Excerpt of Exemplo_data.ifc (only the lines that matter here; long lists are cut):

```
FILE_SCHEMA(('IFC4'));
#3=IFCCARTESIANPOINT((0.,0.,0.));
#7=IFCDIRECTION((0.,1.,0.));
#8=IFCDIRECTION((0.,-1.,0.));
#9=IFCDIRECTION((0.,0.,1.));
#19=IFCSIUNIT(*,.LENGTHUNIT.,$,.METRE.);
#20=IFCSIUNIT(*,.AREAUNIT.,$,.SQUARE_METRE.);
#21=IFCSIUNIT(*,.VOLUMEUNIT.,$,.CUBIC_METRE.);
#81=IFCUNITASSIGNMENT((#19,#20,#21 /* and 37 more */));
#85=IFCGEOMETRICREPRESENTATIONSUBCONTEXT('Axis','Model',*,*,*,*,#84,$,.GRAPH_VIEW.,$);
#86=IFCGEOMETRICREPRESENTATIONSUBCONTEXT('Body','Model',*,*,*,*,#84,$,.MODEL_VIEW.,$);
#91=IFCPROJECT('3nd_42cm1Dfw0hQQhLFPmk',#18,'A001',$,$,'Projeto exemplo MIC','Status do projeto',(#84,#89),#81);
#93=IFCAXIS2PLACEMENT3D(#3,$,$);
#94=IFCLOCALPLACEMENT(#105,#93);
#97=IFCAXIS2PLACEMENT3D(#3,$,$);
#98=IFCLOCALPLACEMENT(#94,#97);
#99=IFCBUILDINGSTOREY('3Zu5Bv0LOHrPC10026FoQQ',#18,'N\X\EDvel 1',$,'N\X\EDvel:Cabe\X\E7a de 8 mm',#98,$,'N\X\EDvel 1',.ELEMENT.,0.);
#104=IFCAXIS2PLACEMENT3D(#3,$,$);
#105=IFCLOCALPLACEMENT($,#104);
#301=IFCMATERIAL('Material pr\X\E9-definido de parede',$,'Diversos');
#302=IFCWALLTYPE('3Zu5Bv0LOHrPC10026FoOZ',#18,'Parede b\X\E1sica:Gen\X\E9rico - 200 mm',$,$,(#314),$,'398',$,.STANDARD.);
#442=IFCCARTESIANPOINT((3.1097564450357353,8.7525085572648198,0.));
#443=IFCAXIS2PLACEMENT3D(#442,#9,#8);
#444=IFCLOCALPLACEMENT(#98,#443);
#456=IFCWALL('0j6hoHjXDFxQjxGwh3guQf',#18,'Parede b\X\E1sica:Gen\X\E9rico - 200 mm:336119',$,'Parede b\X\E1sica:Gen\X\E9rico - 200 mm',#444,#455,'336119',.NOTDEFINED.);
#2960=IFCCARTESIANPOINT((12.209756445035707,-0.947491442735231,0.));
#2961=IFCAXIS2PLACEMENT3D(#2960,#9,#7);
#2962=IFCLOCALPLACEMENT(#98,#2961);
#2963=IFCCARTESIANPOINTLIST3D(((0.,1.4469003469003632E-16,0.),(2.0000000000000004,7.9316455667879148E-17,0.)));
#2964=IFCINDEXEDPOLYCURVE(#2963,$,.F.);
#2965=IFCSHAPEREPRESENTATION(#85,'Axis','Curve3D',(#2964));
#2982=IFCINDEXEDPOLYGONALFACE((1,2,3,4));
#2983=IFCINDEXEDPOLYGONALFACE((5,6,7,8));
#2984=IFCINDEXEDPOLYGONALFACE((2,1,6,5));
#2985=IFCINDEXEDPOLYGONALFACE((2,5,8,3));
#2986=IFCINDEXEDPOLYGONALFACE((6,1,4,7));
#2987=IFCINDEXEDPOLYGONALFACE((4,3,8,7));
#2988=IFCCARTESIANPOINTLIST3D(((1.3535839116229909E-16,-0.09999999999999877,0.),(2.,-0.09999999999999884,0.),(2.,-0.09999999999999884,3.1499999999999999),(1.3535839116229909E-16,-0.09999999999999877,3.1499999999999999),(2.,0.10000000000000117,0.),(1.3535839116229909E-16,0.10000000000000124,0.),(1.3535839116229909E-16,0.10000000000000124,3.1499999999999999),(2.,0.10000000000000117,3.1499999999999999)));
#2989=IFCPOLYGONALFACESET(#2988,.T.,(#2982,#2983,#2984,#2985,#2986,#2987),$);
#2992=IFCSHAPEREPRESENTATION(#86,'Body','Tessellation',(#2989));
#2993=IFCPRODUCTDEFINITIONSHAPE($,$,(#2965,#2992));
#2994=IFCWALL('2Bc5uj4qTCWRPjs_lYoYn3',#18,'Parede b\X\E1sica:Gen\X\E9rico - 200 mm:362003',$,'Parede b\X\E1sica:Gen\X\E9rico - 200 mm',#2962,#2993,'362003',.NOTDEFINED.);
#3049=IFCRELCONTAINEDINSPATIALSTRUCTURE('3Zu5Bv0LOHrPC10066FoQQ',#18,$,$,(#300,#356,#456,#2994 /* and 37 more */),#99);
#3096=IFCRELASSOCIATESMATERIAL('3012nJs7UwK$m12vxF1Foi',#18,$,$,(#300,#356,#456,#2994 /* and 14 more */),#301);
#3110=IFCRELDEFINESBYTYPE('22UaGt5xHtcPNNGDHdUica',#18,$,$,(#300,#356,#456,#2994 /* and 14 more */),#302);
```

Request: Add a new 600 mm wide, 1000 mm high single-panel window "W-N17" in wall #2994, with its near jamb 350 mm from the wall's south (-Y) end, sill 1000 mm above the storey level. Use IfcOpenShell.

```python
import numpy as np
import ifcopenshell
import ifcopenshell.api.feature
import ifcopenshell.api.geometry
import ifcopenshell.api.root
import ifcopenshell.api.spatial
import ifcopenshell.geom
import ifcopenshell.util.element
import ifcopenshell.util.placement
import ifcopenshell.util.representation
import ifcopenshell.util.shape
import ifcopenshell.util.unit

model = ifcopenshell.open("Exemplo_data.ifc")
unit_scale = ifcopenshell.util.unit.calculate_unit_scale(model)
settings = ifcopenshell.geom.settings()


def volume(element):
    """Net volume in cubic metres, openings subtracted."""
    shape = ifcopenshell.geom.create_shape(settings, element)
    return ifcopenshell.util.shape.get_volume(shape.geometry)


wall = model.by_guid("2Bc5uj4qTCWRPjs_lYoYn3")
storey = ifcopenshell.util.element.get_container(wall, ifc_class="IfcBuildingStorey")
context = ifcopenshell.util.representation.get_context(model, "Model", "Body", "MODEL_VIEW")
before = volume(wall)

width, height, from_end, sill = 0.6, 1, 0.35, 1  # metres

# The wall runs along its own X axis, and the end named is its -X end.
wall_shape = ifcopenshell.geom.create_shape(settings, wall)
x, y, z = ifcopenshell.util.shape.get_vertices(wall_shape.geometry).T
start = x.min() + from_end
face, thickness = float(y.min()), float(y.max() - y.min())
wall_matrix = ifcopenshell.util.placement.get_local_placement(wall.ObjectPlacement)
level = ifcopenshell.util.placement.get_local_placement(storey.ObjectPlacement)[2, 3]


def in_wall(x, y):
    """Placement at x, y metres in the wall's axes, at sill height."""
    matrix = wall_matrix.copy()
    matrix[:, 3] = wall_matrix @ np.array([x / unit_scale, y / unit_scale, 0.0, 1.0])
    matrix[2, 3] = level + sill / unit_scale
    return matrix


# Opening: a box that overshoots both wall faces by 50 mm.
opening = ifcopenshell.api.root.create_entity(model, ifc_class="IfcOpeningElement", predefined_type="OPENING")
box = ifcopenshell.api.geometry.add_wall_representation(
    model, context=context, length=width, height=height, thickness=thickness + 0.1
)
ifcopenshell.api.geometry.assign_representation(model, product=opening, representation=box)
ifcopenshell.api.geometry.edit_object_placement(model, product=opening, matrix=in_wall(start, face - 0.05), is_si=False)
ifcopenshell.api.feature.add_feature(model, feature=opening, element=wall)

window = ifcopenshell.api.root.create_entity(model, ifc_class="IfcWindow", name="W-N17", predefined_type="WINDOW")
window.OverallWidth, window.OverallHeight = width / unit_scale, height / unit_scale
window.PartitioningType = "SINGLE_PANEL"
body = ifcopenshell.api.geometry.add_window_representation(
    model,
    context=context,
    overall_width=window.OverallWidth,
    overall_height=window.OverallHeight,
    partition_type="SINGLE_PANEL",
)
ifcopenshell.api.geometry.assign_representation(model, product=window, representation=body)
ifcopenshell.api.spatial.assign_container(model, products=[window], relating_structure=storey)
ifcopenshell.api.feature.add_filling(model, opening=opening, element=window)

# Centre the window in the wall's thickness.
ifcopenshell.api.geometry.edit_object_placement(model, product=window, matrix=in_wall(start, face), is_si=False)
window_shape = ifcopenshell.geom.create_shape(settings, window)
depth = ifcopenshell.util.shape.get_vertices(window_shape.geometry)[:, 1]
offset = face + thickness / 2 - (depth.min() + depth.max()) / 2
ifcopenshell.api.geometry.edit_object_placement(model, product=window, matrix=in_wall(start, offset), is_si=False)

after = volume(wall)

print(f"wall volume {before:.3f} -> {after:.3f} m3")

model.write("Exemplo_data_edited.ifc")
```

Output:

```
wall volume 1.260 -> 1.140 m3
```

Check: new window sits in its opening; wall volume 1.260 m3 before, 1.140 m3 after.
